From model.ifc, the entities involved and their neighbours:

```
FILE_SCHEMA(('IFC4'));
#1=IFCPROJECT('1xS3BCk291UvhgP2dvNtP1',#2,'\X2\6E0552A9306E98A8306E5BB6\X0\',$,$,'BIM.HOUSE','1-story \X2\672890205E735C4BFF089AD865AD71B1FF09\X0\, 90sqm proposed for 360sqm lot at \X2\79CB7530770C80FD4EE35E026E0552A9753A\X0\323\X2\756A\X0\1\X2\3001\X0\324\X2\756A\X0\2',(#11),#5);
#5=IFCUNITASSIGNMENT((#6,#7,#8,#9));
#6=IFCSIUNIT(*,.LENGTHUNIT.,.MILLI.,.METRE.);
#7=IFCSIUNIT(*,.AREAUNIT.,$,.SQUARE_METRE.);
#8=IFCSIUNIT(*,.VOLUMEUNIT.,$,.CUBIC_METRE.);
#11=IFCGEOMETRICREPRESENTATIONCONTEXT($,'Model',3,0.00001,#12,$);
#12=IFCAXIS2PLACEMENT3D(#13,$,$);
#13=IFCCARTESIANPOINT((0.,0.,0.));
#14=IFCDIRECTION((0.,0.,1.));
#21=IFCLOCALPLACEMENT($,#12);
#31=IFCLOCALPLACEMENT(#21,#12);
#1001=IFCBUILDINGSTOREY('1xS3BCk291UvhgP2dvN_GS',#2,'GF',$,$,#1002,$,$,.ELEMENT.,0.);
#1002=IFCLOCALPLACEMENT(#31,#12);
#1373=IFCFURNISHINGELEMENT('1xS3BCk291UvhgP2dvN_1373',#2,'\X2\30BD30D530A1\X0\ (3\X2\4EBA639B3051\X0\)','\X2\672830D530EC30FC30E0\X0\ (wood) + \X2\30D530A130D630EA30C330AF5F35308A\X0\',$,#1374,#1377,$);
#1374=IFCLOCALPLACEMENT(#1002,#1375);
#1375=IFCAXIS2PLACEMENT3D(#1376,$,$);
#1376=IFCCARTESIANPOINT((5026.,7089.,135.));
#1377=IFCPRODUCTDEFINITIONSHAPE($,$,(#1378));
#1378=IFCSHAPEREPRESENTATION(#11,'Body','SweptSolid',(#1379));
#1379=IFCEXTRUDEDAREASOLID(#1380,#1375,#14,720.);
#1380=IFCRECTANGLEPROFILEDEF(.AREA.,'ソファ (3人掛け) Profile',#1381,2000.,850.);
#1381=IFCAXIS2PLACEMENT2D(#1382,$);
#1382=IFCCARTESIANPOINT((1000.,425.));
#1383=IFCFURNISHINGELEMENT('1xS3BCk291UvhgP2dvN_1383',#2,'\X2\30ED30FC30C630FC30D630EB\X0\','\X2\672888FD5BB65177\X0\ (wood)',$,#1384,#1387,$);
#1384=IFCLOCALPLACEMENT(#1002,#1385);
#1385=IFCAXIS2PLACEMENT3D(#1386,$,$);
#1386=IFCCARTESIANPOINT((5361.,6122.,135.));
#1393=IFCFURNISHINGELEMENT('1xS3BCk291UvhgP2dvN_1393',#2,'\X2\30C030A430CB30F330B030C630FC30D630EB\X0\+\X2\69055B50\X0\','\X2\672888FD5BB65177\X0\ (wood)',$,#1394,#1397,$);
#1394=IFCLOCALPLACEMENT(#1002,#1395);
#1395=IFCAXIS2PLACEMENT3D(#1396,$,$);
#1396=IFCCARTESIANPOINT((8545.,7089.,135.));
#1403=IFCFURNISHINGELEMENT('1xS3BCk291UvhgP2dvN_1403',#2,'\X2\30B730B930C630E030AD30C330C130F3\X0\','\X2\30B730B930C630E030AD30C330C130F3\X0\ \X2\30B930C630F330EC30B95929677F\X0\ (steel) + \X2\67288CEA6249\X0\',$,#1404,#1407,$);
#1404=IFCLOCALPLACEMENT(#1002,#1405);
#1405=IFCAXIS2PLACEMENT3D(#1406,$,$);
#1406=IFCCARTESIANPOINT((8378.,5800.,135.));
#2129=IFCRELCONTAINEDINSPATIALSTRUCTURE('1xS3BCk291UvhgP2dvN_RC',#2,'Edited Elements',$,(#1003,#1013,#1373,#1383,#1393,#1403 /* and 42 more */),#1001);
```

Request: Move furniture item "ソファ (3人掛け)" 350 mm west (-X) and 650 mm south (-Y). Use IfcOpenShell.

```python
import ifcopenshell
import ifcopenshell.api.geometry
import ifcopenshell.util.placement

model = ifcopenshell.open("model.ifc")

item = model.by_guid("1xS3BCk291UvhgP2dvN_1373")
matrix = ifcopenshell.util.placement.get_local_placement(item.ObjectPlacement)
matrix[0, 3] -= 350.0
matrix[1, 3] -= 650.0
ifcopenshell.api.geometry.edit_object_placement(model, product=item, matrix=matrix, is_si=False)

print(ifcopenshell.util.placement.get_local_placement(item.ObjectPlacement).round(3) + 0.0)

model.write("model_edited.ifc")
```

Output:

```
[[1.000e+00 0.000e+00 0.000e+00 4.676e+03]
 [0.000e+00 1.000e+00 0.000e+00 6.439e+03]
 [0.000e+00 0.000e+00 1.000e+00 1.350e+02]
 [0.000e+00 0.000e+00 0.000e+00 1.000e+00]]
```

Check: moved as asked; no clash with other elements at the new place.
